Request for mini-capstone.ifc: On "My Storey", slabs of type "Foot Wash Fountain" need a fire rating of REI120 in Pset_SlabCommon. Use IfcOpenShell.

First a look at what the model holds.

```python
import ifcopenshell
import ifcopenshell.util.element

model = ifcopenshell.open("mini-capstone.ifc")
print(model.schema)
storey = next(s for s in model.by_type("IfcBuildingStorey") if s.Name == "My Storey")
slabs = [e for e in ifcopenshell.util.element.get_decomposition(storey) if e.is_a("IfcSlab")]
seen = {}
for e in slabs:
    element_type = ifcopenshell.util.element.get_type(e)
    key = (element_type.Name if element_type != e and element_type else None, ifcopenshell.util.element.get_pset(e, "Pset_SlabCommon", "FireRating"))
    seen[key] = seen.get(key, 0) + 1
for (name, value), count in sorted(seen.items(), key=str):
    print(count, "x", name, "|", value)
```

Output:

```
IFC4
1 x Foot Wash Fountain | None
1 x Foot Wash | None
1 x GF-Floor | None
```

```python
import ifcopenshell
import ifcopenshell.api.pset
import ifcopenshell.util.element

model = ifcopenshell.open("mini-capstone.ifc")

storey = next(s for s in model.by_type("IfcBuildingStorey") if s.Name == "My Storey")
slabs = [e for e in ifcopenshell.util.element.get_decomposition(storey) if e.is_a("IfcSlab")]

count = 0
for e in slabs:
    element_type = ifcopenshell.util.element.get_type(e)
    if element_type in (None, e) or element_type.Name != "Foot Wash Fountain":
        continue
    # add_pset returns the element's existing set when there is one.
    pset = ifcopenshell.api.pset.add_pset(model, product=e, name="Pset_SlabCommon")
    ifcopenshell.api.pset.edit_pset(model, pset=pset, properties={"FireRating": "REI120"})
    count += 1

print(count, "slabs updated")

model.write("mini-capstone_edited.ifc")
```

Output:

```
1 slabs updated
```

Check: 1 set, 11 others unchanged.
